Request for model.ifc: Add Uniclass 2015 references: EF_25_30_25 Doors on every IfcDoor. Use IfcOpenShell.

First a look at what the model holds.

```python
import ifcopenshell

model = ifcopenshell.open("model.ifc")
print(model.schema)
print("classifications:", [c.Name for c in model.by_type("IfcClassification")])
for ifc_class in ("IfcDoor", "IfcRoof", "IfcStair", "IfcWall", "IfcWindow"):
    print(ifc_class, len(model.by_type(ifc_class)))
```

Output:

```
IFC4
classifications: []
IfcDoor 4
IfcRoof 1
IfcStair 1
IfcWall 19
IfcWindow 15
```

```python
import ifcopenshell
import ifcopenshell.api.classification

model = ifcopenshell.open("model.ifc")

system = ifcopenshell.api.classification.add_classification(model, classification="Uniclass 2015")

codes = {
    "IfcDoor": ("EF_25_30_25", "Doors"),
}
for ifc_class, (code, name) in codes.items():
    products = model.by_type(ifc_class)
    ifcopenshell.api.classification.add_reference(
        model, products=products, classification=system, identification=code, name=name
    )
    print(code, len(products))

model.write("model_updated.ifc")
```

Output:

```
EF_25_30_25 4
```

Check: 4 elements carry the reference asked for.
